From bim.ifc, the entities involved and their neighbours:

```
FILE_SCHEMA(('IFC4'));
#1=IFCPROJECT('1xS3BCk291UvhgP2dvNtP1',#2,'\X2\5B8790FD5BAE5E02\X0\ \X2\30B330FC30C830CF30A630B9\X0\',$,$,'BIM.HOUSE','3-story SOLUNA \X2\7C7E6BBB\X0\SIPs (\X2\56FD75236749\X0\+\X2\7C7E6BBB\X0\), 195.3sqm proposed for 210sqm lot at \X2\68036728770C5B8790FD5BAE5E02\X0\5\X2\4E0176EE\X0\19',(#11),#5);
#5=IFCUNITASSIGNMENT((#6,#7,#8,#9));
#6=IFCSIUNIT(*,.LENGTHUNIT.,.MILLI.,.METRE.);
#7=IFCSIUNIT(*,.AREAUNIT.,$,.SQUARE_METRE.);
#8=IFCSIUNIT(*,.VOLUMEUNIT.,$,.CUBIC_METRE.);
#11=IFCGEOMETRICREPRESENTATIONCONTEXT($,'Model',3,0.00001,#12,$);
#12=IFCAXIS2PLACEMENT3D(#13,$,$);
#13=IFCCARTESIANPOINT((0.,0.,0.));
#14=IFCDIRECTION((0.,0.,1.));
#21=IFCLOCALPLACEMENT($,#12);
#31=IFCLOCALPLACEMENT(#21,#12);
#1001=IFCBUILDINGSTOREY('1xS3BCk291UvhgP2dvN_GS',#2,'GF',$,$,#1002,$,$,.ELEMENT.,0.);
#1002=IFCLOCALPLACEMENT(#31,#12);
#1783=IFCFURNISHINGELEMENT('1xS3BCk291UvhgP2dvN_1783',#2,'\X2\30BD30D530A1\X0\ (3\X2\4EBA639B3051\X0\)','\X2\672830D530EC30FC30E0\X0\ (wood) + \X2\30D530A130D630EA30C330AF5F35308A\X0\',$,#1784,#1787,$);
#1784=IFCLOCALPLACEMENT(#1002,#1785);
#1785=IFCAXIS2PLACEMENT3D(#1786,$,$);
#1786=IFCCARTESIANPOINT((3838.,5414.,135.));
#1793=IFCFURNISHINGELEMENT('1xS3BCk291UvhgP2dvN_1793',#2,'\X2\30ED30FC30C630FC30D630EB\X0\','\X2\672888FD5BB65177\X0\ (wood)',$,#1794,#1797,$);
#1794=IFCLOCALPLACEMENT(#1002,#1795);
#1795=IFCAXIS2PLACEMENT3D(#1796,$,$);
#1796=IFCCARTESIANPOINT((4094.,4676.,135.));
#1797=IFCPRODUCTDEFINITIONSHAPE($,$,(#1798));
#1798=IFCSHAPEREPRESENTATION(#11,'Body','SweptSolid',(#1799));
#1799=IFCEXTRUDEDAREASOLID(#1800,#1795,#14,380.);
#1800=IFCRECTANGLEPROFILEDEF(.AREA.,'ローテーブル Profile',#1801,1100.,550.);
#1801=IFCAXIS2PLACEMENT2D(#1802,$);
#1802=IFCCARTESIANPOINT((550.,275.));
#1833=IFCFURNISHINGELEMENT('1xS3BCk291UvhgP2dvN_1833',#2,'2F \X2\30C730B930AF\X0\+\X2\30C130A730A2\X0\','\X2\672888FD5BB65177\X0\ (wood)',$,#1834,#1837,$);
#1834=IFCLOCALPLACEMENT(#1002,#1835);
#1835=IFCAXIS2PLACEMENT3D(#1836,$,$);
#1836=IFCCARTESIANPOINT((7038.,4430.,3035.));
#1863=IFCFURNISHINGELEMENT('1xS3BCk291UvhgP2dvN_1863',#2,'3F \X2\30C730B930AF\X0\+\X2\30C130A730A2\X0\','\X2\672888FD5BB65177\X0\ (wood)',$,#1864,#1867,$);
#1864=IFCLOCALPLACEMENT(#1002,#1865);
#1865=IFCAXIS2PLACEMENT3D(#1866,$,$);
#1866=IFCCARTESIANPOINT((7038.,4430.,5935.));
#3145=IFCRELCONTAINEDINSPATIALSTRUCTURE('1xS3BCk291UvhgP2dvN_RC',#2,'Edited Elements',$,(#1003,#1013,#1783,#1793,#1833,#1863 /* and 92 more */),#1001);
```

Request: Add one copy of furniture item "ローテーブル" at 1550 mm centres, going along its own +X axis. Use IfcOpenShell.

```python
import ifcopenshell
import ifcopenshell.api.geometry
import ifcopenshell.api.root
import ifcopenshell.util.element
import ifcopenshell.util.placement
import ifcopenshell.util.unit

model = ifcopenshell.open("bim.ifc")
unit_scale = ifcopenshell.util.unit.calculate_unit_scale(model)


def reuse_history(source, copy):
    """copy_class also copies each property set's owner history, people and application; keep the originals."""
    for rel in copy.IsDefinedBy:
        if rel.is_a("IfcRelDefinesByProperties") and (history := rel.RelatingPropertyDefinition.OwnerHistory):
            rel.RelatingPropertyDefinition.OwnerHistory = source.OwnerHistory
            ifcopenshell.util.element.remove_deep2(model, history)


source = model.by_id(1793)
base = ifcopenshell.util.placement.get_local_placement(source.ObjectPlacement)
step = base[:3, 0] * 1.55 / unit_scale

for i in range(1, 2):
    copy = ifcopenshell.api.root.copy_class(model, product=source)
    copy.Representation = ifcopenshell.util.element.copy_deep(
        model, source.Representation, exclude=["IfcGeometricRepresentationContext", "IfcRepresentationMap"]
    )
    reuse_history(source, copy)
    matrix = base.copy()
    matrix[:3, 3] += i * step
    print("added at", matrix[:3, 3].round(3) + 0.0)
    ifcopenshell.api.geometry.edit_object_placement(model, product=copy, matrix=matrix, is_si=False)

model.write("bim_rev.ifc")
```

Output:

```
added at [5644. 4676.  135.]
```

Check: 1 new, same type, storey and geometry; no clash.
